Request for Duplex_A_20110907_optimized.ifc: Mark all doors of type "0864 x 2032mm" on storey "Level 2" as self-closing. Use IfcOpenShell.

First a look at what the model holds.

```python
import ifcopenshell
import ifcopenshell.util.element

model = ifcopenshell.open("Duplex_A_20110907_optimized.ifc")
print(model.schema)
storey = next(s for s in model.by_type("IfcBuildingStorey") if s.Name == "Level 2")
doors = [e for e in ifcopenshell.util.element.get_decomposition(storey) if e.is_a("IfcDoor")]
seen = {}
for e in doors:
    element_type = ifcopenshell.util.element.get_type(e)
    key = (element_type.Name if element_type != e and element_type else None, ifcopenshell.util.element.get_pset(e, "Pset_DoorCommon", "SelfClosing"))
    seen[key] = seen.get(key, 0) + 1
for (name, value), count in sorted(seen.items(), key=str):
    print(count, "x", name, "|", value)
```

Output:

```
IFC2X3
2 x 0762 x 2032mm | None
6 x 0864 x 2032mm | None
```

```python
import ifcopenshell
import ifcopenshell.api.pset
import ifcopenshell.util.element

model = ifcopenshell.open("Duplex_A_20110907_optimized.ifc")

storey = next(s for s in model.by_type("IfcBuildingStorey") if s.Name == "Level 2")
doors = [e for e in ifcopenshell.util.element.get_decomposition(storey) if e.is_a("IfcDoor")]

count = 0
for e in doors:
    element_type = ifcopenshell.util.element.get_type(e)
    if element_type in (None, e) or element_type.Name != "0864 x 2032mm":
        continue
    # add_pset returns the element's existing set when there is one.
    pset = ifcopenshell.api.pset.add_pset(model, product=e, name="Pset_DoorCommon")
    ifcopenshell.api.pset.edit_pset(model, pset=pset, properties={"SelfClosing": True})
    count += 1

print(count, "doors updated")

model.write("Duplex_A_20110907_optimized_updated.ifc")
```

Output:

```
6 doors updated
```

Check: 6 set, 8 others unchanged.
